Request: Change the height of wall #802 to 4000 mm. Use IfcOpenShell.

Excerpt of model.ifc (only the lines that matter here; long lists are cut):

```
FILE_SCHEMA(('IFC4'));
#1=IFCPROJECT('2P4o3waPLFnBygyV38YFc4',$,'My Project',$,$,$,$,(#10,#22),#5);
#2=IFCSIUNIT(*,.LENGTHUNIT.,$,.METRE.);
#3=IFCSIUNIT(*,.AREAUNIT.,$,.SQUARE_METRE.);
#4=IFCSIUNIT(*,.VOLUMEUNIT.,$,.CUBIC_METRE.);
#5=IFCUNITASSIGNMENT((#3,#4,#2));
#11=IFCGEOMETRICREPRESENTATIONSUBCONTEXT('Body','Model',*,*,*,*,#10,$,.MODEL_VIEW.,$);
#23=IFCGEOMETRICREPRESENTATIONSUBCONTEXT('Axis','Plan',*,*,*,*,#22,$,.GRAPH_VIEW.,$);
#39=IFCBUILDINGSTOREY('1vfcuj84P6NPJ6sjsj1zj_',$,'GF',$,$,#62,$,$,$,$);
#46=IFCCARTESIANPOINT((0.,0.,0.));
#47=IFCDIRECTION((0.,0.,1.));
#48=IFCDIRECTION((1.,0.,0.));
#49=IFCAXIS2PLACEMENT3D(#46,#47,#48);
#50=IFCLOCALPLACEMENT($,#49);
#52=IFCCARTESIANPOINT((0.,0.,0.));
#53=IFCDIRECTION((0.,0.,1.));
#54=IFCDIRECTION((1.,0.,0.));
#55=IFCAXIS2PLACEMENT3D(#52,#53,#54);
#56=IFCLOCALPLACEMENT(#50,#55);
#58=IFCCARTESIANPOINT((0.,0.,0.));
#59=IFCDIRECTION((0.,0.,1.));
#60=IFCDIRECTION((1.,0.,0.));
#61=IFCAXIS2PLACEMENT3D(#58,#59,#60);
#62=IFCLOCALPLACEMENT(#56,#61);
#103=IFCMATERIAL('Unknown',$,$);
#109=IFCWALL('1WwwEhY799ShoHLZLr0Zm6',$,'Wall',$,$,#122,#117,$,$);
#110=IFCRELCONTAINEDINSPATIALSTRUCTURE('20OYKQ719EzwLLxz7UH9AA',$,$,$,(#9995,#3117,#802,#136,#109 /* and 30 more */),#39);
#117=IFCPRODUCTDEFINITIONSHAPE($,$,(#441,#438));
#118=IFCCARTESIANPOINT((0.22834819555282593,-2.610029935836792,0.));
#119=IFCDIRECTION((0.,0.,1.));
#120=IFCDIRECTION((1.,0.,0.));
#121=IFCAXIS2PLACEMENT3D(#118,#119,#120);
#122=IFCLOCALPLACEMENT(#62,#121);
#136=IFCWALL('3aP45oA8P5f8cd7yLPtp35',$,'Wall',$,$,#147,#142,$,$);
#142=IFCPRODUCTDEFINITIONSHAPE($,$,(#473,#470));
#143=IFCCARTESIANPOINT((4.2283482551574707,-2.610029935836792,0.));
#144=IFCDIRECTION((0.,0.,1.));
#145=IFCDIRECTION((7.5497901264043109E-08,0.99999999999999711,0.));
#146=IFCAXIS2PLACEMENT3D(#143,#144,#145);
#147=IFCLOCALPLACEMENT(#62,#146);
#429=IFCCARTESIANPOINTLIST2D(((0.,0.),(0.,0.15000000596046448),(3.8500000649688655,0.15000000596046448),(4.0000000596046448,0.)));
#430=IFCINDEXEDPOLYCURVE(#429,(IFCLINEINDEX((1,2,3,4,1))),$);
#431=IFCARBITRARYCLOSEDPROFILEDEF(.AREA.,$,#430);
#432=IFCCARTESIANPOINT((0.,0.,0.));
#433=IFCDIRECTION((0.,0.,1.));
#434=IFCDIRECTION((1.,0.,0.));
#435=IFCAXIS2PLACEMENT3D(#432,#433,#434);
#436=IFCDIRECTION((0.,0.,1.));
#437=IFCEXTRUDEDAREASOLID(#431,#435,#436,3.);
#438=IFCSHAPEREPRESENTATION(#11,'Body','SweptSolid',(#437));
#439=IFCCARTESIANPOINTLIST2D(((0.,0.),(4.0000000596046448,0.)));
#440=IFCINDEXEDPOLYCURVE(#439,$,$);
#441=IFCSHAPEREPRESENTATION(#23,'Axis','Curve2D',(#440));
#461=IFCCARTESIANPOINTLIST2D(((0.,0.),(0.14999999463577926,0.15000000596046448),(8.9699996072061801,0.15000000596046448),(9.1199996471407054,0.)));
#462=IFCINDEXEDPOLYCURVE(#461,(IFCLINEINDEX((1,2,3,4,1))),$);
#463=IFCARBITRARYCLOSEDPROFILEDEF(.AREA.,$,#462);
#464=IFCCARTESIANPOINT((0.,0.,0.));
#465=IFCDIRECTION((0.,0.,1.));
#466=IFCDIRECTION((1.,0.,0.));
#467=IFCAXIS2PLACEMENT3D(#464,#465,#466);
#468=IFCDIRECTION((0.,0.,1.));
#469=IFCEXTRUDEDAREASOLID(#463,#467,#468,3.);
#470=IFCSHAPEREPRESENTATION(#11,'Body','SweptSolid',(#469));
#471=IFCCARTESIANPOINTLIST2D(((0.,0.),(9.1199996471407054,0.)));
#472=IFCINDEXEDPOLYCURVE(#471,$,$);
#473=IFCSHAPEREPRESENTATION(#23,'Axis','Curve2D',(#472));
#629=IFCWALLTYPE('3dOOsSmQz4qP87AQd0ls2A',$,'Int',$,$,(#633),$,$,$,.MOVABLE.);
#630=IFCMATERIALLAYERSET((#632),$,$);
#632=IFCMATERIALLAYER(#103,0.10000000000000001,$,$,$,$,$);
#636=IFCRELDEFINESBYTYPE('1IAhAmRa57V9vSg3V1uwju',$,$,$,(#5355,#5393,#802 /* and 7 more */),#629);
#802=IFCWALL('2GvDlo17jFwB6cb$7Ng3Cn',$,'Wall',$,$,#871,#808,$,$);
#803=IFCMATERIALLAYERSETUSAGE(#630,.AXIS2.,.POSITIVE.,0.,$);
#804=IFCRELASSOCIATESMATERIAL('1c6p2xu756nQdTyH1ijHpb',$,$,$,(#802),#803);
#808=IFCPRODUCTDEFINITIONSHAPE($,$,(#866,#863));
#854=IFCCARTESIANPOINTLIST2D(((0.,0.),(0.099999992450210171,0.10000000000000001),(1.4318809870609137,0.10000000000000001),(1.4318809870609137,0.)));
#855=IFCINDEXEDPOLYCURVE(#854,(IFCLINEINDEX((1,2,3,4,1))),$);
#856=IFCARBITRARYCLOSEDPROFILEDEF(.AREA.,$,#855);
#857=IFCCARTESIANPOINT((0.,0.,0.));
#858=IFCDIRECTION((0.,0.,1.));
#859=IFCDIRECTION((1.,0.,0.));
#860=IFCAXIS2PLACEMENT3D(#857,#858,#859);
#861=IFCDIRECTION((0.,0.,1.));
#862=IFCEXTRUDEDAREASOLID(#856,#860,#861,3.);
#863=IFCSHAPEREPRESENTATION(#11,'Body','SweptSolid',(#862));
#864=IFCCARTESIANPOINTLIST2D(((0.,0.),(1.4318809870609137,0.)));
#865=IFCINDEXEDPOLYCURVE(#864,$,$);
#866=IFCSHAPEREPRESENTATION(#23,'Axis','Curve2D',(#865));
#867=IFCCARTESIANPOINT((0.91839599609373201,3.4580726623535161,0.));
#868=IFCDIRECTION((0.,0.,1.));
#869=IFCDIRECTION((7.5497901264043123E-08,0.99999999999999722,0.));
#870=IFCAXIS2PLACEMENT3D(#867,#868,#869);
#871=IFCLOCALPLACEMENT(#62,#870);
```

```python
import ifcopenshell
import ifcopenshell.geom
import ifcopenshell.util.representation
import ifcopenshell.util.shape

model = ifcopenshell.open("model.ifc")
settings = ifcopenshell.geom.settings()


def volume(element):
    """Net volume in cubic metres, openings subtracted."""
    shape = ifcopenshell.geom.create_shape(settings, element)
    return ifcopenshell.util.shape.get_volume(shape.geometry)


wall = model.by_guid("2GvDlo17jFwB6cb$7Ng3Cn")
before = volume(wall)

body = ifcopenshell.util.representation.get_representation(wall, "Model", "Body")
solid = body.Items[0]
old_height = solid.Depth
solid.Depth = 4.0
after = volume(wall)

print(f"height {old_height:g} -> {solid.Depth:g}, volume {before:.3f} -> {after:.3f} m3")

model.write("model_updated.ifc")
```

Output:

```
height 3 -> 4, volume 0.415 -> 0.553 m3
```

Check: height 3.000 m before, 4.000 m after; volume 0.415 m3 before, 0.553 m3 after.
